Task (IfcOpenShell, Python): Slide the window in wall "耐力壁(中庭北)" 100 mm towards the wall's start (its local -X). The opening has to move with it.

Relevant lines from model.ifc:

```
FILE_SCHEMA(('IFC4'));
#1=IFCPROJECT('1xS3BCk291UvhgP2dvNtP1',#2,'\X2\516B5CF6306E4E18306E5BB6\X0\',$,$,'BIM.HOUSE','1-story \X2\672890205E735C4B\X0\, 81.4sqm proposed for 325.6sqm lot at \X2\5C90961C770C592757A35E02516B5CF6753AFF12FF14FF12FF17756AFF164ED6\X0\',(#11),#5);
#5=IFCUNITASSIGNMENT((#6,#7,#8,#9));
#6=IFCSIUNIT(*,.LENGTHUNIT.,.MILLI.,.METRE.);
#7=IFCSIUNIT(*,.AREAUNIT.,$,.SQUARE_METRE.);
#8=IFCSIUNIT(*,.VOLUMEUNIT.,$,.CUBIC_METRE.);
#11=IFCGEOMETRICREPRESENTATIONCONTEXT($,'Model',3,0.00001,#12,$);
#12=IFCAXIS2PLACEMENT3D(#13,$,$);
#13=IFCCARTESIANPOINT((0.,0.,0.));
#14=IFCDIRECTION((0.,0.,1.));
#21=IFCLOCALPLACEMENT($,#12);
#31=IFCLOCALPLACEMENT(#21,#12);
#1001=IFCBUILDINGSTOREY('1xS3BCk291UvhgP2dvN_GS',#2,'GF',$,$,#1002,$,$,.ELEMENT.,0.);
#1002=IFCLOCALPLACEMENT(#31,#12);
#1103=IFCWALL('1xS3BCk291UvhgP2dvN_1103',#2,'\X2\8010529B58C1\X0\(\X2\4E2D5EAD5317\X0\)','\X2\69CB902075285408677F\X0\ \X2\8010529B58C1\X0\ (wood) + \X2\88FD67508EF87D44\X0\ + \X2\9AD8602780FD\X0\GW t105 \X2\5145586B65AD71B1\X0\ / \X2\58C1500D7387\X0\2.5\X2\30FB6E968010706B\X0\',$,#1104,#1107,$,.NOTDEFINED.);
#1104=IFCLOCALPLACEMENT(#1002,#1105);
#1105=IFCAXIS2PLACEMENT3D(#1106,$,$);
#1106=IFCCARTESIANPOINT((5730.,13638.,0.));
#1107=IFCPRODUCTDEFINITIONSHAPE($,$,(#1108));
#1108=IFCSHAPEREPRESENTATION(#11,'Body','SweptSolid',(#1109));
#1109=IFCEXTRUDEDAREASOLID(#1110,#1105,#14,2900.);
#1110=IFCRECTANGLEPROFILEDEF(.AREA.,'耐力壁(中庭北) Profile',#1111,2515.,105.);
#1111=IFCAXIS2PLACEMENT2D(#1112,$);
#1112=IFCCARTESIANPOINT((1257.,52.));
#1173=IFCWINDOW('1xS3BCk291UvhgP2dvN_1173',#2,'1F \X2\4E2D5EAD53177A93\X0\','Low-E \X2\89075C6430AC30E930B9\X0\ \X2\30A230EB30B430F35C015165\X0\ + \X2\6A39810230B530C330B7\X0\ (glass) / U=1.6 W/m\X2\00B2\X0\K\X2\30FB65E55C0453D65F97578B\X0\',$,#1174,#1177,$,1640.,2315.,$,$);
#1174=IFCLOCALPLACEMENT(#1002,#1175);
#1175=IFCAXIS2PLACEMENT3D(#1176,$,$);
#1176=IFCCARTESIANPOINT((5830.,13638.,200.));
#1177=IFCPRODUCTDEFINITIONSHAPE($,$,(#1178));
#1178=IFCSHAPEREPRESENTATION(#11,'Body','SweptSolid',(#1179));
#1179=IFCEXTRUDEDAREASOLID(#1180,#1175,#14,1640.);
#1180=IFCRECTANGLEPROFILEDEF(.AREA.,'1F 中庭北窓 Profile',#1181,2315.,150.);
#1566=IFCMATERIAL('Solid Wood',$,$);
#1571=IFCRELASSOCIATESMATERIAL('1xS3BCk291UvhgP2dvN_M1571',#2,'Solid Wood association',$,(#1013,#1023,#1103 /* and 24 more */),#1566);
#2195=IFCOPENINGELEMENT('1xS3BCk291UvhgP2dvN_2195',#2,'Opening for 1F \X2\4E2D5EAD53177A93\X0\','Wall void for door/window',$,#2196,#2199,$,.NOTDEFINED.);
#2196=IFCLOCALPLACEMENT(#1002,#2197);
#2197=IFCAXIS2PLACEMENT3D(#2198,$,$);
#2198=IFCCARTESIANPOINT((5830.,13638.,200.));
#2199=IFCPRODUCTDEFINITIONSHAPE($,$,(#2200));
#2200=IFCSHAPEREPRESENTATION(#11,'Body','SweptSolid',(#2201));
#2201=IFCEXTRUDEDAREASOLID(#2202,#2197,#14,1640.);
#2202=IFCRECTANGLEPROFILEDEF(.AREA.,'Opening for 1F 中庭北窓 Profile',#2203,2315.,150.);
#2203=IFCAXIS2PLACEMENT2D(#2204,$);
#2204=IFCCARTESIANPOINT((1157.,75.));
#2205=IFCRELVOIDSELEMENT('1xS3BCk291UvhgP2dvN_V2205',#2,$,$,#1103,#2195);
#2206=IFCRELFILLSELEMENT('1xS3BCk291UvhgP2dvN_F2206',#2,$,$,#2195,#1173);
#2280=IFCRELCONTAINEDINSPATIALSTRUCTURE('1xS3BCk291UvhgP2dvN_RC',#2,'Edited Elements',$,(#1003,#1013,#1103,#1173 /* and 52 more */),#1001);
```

```python
import ifcopenshell
import ifcopenshell.api.geometry
import ifcopenshell.util.placement
import ifcopenshell.util.unit

model = ifcopenshell.open("model.ifc")
unit_scale = ifcopenshell.util.unit.calculate_unit_scale(model)

window = model.by_id(1173)
opening = window.FillsVoids[0].RelatingOpeningElement
wall = opening.VoidsElements[0].RelatingBuildingElement

wall_matrix = ifcopenshell.util.placement.get_local_placement(wall.ObjectPlacement)
shift = wall_matrix[:3, 0] * -0.1 / unit_scale
before = ifcopenshell.util.placement.get_local_placement(window.ObjectPlacement)[:3, 3].copy()

# The window is not placed relative to its opening, so move both.
for product in (opening, window):
    matrix = ifcopenshell.util.placement.get_local_placement(product.ObjectPlacement)
    matrix[:3, 3] += shift
    ifcopenshell.api.geometry.edit_object_placement(model, product=product, matrix=matrix, is_si=False)

after = ifcopenshell.util.placement.get_local_placement(window.ObjectPlacement)[:3, 3]
print("window moved by", (after - before).round(3) + 0.0)

model.write("model_edited.ifc")
```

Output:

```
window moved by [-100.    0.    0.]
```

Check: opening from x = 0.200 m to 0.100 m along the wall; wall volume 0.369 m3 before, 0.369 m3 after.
